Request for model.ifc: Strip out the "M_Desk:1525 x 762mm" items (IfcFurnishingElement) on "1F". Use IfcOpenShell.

First a look at what the model holds.

```python
import ifcopenshell
import ifcopenshell.util.element

model = ifcopenshell.open("model.ifc")
print(model.schema)
storey = next(s for s in model.by_type("IfcBuildingStorey") if s.Name == "1F")
furniture = [e for e in ifcopenshell.util.element.get_decomposition(storey) if e.is_a("IfcFurnishingElement")]
seen = {}
for e in furniture:
    element_type = ifcopenshell.util.element.get_type(e)
    name = element_type.Name if element_type not in (None, e) else None
    seen[name] = seen.get(name, 0) + 1
for name, count in sorted(seen.items(), key=str):
    print(count, "x", name)
```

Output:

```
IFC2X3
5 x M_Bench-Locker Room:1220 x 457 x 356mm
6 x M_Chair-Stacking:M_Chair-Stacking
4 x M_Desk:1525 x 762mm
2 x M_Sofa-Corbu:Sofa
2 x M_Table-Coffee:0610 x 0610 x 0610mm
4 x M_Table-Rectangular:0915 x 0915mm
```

```python
import ifcopenshell
import ifcopenshell.api.root
import ifcopenshell.util.element

model = ifcopenshell.open("model.ifc")

storey = next(s for s in model.by_type("IfcBuildingStorey") if s.Name == "1F")
furniture = [e for e in ifcopenshell.util.element.get_decomposition(storey) if e.is_a("IfcFurnishingElement")]
targets = [e for e in furniture if (t := ifcopenshell.util.element.get_type(e)) not in (None, e) and t.Name == "M_Desk:1525 x 762mm"]

for e in targets:
    ifcopenshell.api.root.remove_product(model, product=e)
print(len(targets), "removed")

model.write("model_v2.ifc")
```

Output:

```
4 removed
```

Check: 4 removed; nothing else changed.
